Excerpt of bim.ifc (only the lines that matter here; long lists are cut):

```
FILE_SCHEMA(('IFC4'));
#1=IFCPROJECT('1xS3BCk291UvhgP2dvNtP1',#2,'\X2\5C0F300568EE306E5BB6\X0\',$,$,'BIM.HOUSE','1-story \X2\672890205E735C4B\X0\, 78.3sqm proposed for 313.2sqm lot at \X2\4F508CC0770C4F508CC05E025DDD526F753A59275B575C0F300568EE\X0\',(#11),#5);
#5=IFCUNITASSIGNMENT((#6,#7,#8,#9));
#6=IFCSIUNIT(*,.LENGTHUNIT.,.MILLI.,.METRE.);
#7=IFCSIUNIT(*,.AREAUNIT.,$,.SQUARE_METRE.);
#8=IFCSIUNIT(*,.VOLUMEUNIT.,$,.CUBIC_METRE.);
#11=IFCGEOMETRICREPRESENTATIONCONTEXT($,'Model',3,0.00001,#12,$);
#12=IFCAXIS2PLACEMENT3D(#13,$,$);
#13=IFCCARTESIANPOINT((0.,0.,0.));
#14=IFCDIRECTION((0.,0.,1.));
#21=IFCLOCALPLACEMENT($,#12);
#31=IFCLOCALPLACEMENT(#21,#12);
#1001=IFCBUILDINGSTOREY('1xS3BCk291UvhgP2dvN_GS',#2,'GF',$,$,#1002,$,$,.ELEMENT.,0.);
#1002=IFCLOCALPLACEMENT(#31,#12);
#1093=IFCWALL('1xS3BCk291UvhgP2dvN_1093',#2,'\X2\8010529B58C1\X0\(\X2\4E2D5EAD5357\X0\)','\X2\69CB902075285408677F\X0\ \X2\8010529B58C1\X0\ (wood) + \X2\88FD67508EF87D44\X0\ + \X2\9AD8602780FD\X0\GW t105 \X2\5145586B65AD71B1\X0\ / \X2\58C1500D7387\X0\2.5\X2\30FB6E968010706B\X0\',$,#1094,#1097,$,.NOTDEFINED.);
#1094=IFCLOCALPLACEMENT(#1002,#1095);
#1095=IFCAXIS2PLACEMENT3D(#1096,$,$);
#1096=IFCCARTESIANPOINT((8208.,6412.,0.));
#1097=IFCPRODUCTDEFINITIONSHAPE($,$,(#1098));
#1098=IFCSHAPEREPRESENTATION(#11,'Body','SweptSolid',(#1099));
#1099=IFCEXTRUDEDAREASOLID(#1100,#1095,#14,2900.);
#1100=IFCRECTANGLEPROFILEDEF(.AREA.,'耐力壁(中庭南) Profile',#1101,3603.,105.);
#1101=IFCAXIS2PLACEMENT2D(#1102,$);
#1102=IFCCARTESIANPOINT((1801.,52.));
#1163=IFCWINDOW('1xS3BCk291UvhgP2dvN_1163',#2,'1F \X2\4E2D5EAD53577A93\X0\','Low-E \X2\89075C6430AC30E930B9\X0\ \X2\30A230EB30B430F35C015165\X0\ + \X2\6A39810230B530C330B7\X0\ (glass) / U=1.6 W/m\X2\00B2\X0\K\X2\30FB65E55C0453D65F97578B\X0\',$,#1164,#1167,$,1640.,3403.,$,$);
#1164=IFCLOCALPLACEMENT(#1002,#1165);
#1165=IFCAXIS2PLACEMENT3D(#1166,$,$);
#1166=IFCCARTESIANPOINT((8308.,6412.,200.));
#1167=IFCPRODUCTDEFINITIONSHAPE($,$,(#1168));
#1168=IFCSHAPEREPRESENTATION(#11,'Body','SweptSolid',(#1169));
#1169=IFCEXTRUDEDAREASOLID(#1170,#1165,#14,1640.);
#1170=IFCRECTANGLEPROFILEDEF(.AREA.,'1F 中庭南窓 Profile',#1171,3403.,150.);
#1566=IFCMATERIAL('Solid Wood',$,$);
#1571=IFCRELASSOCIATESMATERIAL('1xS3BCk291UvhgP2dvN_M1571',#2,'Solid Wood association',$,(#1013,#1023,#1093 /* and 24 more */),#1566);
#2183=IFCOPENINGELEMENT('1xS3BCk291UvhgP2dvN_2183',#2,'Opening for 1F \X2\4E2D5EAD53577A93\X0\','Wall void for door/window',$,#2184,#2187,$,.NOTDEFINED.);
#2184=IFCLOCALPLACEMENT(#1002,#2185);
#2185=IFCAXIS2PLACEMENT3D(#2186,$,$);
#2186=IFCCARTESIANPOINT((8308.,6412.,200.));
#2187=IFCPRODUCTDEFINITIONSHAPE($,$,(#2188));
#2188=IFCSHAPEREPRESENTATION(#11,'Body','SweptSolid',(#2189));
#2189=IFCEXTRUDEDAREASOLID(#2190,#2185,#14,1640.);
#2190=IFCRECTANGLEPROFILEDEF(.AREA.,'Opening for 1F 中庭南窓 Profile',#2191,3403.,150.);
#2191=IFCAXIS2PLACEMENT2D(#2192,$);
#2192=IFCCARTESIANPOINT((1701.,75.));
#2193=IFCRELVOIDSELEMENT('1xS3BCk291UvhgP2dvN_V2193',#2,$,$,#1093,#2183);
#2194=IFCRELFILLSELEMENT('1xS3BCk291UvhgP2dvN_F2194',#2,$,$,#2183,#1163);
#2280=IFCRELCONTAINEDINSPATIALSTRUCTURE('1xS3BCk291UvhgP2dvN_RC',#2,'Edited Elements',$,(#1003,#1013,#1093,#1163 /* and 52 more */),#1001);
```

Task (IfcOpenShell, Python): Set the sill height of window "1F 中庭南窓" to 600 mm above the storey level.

```python
import numpy as np
import ifcopenshell
import ifcopenshell.api.geometry
import ifcopenshell.geom
import ifcopenshell.util.element
import ifcopenshell.util.placement
import ifcopenshell.util.shape
import ifcopenshell.util.unit

model = ifcopenshell.open("bim.ifc")
unit_scale = ifcopenshell.util.unit.calculate_unit_scale(model)

window = model.by_guid("1xS3BCk291UvhgP2dvN_1163")
opening = window.FillsVoids[0].RelatingOpeningElement
storey = ifcopenshell.util.element.get_container(window, ifc_class="IfcBuildingStorey")
level = ifcopenshell.util.placement.get_local_placement(storey.ObjectPlacement)[2, 3]

# The opening's origin need not be at the sill, so measure its lowest point.
shape = ifcopenshell.geom.create_shape(ifcopenshell.geom.settings(), opening)
bottom = ifcopenshell.util.shape.get_shape_bottom_elevation(shape, shape.geometry) / unit_scale
dz = level + 600.0 - bottom

shift = np.array([0.0, 0.0, dz])
# The window is not placed relative to its opening, so move both.
for product in (opening, window):
    matrix = ifcopenshell.util.placement.get_local_placement(product.ObjectPlacement)
    matrix[:3, 3] += shift
    ifcopenshell.api.geometry.edit_object_placement(model, product=product, matrix=matrix, is_si=False)

print(f"moved by {dz * unit_scale:+.3f} m")

model.write("bim_updated.ifc")
```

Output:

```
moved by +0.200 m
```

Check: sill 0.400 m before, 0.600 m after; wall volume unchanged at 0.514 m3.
